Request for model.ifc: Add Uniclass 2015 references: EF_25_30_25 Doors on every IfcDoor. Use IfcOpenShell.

First a look at what the model holds.

```python
import ifcopenshell

model = ifcopenshell.open("model.ifc")
print(model.schema)
print("classifications:", [c.Name for c in model.by_type("IfcClassification")])
for ifc_class in ("IfcDoor", "IfcRoof", "IfcStair", "IfcWall", "IfcWindow"):
    print(ifc_class, len(model.by_type(ifc_class)))
```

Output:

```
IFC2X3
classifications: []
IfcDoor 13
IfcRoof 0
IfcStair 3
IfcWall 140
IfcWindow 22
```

```python
import ifcopenshell
import ifcopenshell.api.classification

model = ifcopenshell.open("model.ifc")

# IFC2X3 requires Source and Edition and has no link from the project to the system.
system = model.create_entity("IfcClassification", Source="NBS", Edition="2015", Name="Uniclass 2015")

codes = {
    "IfcDoor": ("EF_25_30_25", "Doors"),
}
for ifc_class, (code, name) in codes.items():
    products = model.by_type(ifc_class)
    ifcopenshell.api.classification.add_reference(
        model, products=products, classification=system, identification=code, name=name
    )
    print(code, len(products))

model.write("model_rev.ifc")
```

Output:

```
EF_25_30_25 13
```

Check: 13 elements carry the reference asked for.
